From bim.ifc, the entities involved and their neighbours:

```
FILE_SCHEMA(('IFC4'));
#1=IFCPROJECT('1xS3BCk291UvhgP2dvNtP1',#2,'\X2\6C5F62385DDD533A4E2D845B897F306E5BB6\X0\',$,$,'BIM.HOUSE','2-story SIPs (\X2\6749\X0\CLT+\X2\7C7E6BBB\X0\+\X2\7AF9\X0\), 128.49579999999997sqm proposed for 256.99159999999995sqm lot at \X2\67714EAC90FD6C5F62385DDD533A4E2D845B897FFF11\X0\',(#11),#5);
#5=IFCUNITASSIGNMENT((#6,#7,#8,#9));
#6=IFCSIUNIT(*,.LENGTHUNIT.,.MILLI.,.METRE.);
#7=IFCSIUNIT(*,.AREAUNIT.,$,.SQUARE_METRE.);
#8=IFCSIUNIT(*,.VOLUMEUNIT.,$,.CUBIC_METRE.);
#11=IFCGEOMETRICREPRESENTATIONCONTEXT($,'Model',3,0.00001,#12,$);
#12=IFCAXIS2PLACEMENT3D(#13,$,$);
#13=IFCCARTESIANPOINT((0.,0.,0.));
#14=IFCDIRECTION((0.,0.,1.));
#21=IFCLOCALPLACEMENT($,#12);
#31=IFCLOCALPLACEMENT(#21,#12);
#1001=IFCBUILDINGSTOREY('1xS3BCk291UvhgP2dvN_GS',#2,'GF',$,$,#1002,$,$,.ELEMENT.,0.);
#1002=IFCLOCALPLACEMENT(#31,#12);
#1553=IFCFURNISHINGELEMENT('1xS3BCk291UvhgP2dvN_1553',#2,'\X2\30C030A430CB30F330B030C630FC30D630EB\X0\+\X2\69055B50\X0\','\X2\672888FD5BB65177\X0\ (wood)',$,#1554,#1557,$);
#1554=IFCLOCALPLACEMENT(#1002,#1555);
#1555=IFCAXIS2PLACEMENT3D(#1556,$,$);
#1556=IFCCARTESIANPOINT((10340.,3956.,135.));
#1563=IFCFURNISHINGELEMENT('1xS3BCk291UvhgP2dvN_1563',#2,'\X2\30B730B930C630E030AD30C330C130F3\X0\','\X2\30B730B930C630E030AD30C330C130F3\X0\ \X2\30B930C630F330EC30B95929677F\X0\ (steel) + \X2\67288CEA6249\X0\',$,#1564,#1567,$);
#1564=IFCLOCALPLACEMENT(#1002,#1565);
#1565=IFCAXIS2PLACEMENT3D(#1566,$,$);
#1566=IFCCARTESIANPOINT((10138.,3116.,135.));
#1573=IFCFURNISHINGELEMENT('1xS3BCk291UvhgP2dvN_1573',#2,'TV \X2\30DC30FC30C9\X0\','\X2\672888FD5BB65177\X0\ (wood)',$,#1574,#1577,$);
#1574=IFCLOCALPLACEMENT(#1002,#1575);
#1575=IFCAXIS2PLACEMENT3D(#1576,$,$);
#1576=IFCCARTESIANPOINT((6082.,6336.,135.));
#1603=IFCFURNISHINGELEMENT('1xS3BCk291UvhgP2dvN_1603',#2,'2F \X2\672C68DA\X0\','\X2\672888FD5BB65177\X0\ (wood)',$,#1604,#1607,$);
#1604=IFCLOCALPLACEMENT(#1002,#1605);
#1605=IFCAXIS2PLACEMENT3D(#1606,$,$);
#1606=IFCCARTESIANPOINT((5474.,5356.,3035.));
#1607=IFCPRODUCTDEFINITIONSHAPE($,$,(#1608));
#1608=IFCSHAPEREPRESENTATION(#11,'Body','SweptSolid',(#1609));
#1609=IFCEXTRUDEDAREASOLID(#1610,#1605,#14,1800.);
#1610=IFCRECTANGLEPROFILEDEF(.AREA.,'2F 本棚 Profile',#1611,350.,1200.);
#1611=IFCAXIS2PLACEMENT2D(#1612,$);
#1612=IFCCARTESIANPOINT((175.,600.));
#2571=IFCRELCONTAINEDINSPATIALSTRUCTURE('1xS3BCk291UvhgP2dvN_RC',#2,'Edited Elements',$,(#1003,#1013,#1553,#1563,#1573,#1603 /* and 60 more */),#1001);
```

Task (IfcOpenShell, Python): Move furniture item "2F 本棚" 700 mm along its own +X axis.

```python
import ifcopenshell
import ifcopenshell.api.geometry
import ifcopenshell.util.placement
import ifcopenshell.util.unit

model = ifcopenshell.open("bim.ifc")
unit_scale = ifcopenshell.util.unit.calculate_unit_scale(model)

item = model.by_id(1603)
matrix = ifcopenshell.util.placement.get_local_placement(item.ObjectPlacement)
matrix[:3, 3] += matrix[:3, 0] * 0.7 / unit_scale
ifcopenshell.api.geometry.edit_object_placement(model, product=item, matrix=matrix, is_si=False)

print(ifcopenshell.util.placement.get_local_placement(item.ObjectPlacement).round(3) + 0.0)

model.write("bim_edited.ifc")
```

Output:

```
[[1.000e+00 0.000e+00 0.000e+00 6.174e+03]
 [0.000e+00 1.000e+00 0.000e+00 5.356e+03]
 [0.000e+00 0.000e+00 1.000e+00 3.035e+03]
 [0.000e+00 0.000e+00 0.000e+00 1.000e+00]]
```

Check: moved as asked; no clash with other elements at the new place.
